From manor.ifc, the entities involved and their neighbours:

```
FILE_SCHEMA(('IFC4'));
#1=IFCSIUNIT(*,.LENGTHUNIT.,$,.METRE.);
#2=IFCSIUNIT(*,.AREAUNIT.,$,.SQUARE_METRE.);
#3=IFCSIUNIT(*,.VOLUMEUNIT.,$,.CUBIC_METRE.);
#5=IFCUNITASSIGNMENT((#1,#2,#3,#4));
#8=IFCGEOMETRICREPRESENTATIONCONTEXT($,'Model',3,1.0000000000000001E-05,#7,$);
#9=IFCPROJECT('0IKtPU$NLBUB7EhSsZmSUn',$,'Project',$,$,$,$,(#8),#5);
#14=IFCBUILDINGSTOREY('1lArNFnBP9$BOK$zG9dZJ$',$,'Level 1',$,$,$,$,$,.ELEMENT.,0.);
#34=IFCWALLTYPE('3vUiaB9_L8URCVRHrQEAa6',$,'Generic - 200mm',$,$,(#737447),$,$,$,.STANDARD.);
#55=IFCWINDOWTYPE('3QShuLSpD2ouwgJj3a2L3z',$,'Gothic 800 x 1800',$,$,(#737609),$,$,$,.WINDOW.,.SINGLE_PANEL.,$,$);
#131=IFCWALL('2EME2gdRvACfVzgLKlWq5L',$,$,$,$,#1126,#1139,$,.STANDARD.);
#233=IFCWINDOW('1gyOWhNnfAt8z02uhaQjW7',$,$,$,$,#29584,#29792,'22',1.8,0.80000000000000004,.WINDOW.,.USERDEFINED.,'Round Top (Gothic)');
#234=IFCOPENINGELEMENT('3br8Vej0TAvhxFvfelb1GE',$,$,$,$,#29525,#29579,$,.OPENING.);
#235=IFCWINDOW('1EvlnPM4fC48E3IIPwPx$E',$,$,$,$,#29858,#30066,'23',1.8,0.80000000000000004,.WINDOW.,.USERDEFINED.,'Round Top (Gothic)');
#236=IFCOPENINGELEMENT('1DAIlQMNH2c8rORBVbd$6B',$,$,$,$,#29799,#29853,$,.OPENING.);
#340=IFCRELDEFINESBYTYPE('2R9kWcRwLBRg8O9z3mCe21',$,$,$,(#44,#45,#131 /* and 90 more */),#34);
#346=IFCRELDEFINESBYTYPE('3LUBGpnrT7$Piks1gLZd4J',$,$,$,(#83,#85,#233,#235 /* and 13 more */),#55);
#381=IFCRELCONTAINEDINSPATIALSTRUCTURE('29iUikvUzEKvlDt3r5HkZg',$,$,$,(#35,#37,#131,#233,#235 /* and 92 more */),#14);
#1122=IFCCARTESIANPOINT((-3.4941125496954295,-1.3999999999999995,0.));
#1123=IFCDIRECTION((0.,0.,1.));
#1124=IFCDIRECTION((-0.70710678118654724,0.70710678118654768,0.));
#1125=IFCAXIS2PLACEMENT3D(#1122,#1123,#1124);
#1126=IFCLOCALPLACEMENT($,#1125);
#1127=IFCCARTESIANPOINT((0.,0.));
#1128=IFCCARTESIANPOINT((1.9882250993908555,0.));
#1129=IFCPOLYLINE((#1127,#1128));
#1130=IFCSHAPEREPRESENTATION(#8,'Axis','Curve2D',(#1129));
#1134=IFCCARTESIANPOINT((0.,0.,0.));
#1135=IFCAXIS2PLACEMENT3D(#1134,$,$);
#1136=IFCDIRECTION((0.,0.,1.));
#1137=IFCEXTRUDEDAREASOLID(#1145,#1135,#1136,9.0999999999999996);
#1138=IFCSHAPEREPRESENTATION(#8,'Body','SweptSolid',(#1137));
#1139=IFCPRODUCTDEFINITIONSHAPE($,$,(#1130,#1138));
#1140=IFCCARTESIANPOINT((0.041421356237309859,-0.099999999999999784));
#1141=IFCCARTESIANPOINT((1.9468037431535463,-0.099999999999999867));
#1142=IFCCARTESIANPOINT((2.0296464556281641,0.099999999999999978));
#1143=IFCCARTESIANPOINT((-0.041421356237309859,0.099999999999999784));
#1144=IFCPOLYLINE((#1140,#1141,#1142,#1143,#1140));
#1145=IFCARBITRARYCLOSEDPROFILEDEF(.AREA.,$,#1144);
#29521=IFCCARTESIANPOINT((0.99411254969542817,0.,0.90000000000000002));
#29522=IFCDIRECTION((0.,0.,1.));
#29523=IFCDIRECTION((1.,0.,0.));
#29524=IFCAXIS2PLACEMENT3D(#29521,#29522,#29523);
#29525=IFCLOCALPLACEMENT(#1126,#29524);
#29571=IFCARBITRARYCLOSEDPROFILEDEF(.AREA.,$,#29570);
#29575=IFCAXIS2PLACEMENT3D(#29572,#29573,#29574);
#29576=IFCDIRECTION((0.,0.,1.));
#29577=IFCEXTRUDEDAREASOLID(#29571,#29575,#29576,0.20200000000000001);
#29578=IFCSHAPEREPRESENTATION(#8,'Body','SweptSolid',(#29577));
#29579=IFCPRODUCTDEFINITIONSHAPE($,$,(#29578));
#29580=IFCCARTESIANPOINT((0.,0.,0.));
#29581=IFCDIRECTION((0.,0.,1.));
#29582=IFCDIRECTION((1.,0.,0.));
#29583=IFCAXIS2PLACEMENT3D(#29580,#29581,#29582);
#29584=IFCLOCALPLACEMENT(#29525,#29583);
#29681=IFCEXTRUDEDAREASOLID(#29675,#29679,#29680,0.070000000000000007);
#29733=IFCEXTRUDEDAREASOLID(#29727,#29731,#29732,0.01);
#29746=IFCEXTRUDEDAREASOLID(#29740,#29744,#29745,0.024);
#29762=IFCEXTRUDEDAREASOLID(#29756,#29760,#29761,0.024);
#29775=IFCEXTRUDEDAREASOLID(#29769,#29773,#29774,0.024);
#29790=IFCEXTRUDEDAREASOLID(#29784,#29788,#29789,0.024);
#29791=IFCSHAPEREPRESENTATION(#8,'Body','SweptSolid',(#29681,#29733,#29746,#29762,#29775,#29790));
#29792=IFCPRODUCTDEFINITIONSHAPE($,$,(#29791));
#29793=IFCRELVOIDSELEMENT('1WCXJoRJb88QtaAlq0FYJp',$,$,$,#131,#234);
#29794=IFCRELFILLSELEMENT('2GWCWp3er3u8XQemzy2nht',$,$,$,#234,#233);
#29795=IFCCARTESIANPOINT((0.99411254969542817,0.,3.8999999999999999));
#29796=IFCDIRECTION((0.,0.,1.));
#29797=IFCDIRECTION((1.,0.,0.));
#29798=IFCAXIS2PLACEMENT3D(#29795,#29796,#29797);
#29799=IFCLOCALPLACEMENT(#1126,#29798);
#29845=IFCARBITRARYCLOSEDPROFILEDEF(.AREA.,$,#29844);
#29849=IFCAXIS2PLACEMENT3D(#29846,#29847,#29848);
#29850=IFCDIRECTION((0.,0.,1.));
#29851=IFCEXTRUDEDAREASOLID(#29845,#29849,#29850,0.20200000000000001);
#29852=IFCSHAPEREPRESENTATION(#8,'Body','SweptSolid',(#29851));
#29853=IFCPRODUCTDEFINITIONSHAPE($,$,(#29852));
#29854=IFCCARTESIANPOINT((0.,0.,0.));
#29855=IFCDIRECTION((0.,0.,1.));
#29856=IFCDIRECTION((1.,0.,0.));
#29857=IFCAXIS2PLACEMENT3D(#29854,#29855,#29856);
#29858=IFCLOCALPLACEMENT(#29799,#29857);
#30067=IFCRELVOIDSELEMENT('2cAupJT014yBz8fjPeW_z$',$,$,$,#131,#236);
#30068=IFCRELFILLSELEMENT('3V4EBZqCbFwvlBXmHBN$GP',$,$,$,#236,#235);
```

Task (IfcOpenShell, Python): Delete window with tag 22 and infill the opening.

```python
import ifcopenshell
import ifcopenshell.api.feature
import ifcopenshell.api.root
import ifcopenshell.geom
import ifcopenshell.util.shape

model = ifcopenshell.open("manor.ifc")
settings = ifcopenshell.geom.settings()


def volume(element):
    """Net volume in cubic metres, openings subtracted."""
    shape = ifcopenshell.geom.create_shape(settings, element)
    return ifcopenshell.util.shape.get_volume(shape.geometry)


window = model.by_id(233)
opening = window.FillsVoids[0].RelatingOpeningElement
wall = opening.VoidsElements[0].RelatingBuildingElement
before = volume(wall)

ifcopenshell.api.root.remove_product(model, product=window)
ifcopenshell.api.feature.remove_feature(model, feature=opening)

after = volume(wall)

print(f"wall volume {before:.3f} -> {after:.3f} m3")

model.write("manor-out.ifc")
```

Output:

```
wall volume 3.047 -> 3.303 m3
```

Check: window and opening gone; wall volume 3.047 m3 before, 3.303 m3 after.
